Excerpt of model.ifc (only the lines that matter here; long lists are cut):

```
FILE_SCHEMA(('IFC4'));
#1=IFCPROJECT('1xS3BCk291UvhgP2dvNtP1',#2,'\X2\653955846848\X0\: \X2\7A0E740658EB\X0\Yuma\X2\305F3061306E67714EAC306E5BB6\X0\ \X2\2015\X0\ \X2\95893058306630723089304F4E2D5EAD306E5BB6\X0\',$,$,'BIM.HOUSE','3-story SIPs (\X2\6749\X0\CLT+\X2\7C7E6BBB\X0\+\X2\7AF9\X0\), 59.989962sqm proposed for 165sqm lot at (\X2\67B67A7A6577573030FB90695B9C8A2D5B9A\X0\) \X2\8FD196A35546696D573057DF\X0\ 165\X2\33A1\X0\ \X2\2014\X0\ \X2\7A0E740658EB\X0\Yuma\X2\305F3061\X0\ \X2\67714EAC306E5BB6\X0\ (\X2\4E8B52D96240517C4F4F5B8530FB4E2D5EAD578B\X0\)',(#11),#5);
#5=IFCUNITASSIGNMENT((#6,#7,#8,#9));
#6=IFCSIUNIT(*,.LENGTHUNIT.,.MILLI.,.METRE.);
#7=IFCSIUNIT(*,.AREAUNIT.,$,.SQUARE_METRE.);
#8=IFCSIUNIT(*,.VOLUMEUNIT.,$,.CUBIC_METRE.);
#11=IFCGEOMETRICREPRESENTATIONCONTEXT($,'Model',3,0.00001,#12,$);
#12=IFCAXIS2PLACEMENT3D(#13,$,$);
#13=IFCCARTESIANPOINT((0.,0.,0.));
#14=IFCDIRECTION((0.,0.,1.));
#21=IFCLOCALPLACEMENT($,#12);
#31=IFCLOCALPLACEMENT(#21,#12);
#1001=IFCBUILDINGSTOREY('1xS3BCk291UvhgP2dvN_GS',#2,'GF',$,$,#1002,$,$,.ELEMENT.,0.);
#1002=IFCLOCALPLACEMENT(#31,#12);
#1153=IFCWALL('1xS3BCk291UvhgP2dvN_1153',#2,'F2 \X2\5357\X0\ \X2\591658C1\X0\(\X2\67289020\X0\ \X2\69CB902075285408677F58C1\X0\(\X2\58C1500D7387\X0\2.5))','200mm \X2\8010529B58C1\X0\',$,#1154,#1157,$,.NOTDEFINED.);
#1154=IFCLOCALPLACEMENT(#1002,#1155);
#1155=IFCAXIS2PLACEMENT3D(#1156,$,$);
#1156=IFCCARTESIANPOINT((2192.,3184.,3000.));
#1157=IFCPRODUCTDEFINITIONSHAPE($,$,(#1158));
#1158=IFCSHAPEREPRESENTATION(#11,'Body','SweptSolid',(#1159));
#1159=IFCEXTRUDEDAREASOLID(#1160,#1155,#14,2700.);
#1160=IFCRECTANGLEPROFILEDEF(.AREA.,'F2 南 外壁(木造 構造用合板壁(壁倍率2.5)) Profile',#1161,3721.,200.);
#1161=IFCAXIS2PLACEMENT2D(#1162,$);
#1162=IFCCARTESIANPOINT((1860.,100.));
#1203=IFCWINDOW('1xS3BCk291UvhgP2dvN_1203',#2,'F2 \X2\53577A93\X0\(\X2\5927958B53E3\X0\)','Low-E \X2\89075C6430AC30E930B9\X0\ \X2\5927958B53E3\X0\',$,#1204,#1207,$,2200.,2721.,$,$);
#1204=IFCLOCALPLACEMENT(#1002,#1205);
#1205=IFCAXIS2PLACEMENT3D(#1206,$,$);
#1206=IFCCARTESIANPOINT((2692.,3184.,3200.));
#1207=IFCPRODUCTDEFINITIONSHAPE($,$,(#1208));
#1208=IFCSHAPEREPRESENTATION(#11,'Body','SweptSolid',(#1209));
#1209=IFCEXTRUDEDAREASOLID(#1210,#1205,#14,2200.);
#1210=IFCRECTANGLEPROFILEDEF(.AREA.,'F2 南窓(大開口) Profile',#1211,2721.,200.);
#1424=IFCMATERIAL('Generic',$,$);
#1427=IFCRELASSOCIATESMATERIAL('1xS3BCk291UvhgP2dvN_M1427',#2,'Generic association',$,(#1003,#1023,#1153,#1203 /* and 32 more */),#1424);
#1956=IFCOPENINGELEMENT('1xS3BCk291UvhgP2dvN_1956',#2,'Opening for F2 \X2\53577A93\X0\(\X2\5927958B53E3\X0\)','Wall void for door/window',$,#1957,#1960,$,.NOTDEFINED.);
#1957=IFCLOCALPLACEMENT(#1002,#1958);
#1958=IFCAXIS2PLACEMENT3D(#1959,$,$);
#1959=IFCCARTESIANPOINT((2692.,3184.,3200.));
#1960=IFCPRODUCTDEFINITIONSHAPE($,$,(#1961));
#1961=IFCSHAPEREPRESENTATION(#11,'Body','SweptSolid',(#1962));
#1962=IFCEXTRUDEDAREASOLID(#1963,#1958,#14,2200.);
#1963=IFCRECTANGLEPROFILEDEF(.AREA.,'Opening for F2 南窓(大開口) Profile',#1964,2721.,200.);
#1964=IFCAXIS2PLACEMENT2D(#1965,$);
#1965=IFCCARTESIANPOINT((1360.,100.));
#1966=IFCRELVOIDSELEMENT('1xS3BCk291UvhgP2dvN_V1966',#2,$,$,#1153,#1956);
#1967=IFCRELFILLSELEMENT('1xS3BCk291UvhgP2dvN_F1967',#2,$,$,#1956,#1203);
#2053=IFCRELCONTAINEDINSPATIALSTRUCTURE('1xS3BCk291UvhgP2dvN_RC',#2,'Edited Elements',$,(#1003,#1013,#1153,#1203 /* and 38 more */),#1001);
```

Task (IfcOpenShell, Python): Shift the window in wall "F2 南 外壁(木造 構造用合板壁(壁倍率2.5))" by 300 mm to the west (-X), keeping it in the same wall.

```python
import ifcopenshell
import ifcopenshell.api.geometry
import ifcopenshell.util.placement
import ifcopenshell.util.unit

model = ifcopenshell.open("model.ifc")
unit_scale = ifcopenshell.util.unit.calculate_unit_scale(model)

window = model.by_guid("1xS3BCk291UvhgP2dvN_1203")
opening = window.FillsVoids[0].RelatingOpeningElement
wall = opening.VoidsElements[0].RelatingBuildingElement

wall_matrix = ifcopenshell.util.placement.get_local_placement(wall.ObjectPlacement)
shift = wall_matrix[:3, 0] * -0.3 / unit_scale
before = ifcopenshell.util.placement.get_local_placement(window.ObjectPlacement)[:3, 3].copy()

# The window is not placed relative to its opening, so move both.
for product in (opening, window):
    matrix = ifcopenshell.util.placement.get_local_placement(product.ObjectPlacement)
    matrix[:3, 3] += shift
    ifcopenshell.api.geometry.edit_object_placement(model, product=product, matrix=matrix, is_si=False)

after = ifcopenshell.util.placement.get_local_placement(window.ObjectPlacement)[:3, 3]
print("window moved by", (after - before).round(3) + 0.0)

model.write("model_v2.ifc")
```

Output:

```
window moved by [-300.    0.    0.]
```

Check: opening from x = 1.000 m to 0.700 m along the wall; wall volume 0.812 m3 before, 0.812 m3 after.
